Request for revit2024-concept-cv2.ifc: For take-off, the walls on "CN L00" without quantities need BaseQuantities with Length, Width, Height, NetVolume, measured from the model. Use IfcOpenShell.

First a look at what the model holds.

```python
import ifcopenshell
import ifcopenshell.util.element
import ifcopenshell.util.unit

model = ifcopenshell.open("revit2024-concept-cv2.ifc")
print(model.schema)
for unit_type in ("LENGTHUNIT", "AREAUNIT", "VOLUMEUNIT"):
    print(unit_type, ifcopenshell.util.unit.calculate_unit_scale(model, unit_type))
storey = next(s for s in model.by_type("IfcBuildingStorey") if s.Name == "CN L00")
walls = [e for e in ifcopenshell.util.element.get_decomposition(storey) if e.is_a("IfcWall")]
for e in sorted(walls, key=lambda e: e.id()):
    print(e.id(), e.is_a(), e.Name, list(ifcopenshell.util.element.get_psets(e, qtos_only=True)), sep=" | ")
```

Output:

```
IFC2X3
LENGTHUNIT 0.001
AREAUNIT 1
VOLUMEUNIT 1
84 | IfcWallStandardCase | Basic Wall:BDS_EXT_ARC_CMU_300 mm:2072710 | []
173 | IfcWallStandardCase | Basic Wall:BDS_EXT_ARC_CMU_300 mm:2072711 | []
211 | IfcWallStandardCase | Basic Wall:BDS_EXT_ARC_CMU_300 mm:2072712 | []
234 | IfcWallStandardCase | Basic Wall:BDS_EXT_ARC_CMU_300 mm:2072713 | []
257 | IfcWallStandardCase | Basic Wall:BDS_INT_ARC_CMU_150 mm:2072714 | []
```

```python
import ifcopenshell
import ifcopenshell.api.pset
import ifcopenshell.geom
import ifcopenshell.util.element
import ifcopenshell.util.shape
import ifcopenshell.util.unit

model = ifcopenshell.open("revit2024-concept-cv2.ifc")
unit_scale = ifcopenshell.util.unit.calculate_unit_scale(model)
volume_scale = ifcopenshell.util.unit.calculate_unit_scale(model, "VOLUMEUNIT")
settings = ifcopenshell.geom.settings()

storey = next(s for s in model.by_type("IfcBuildingStorey") if s.Name == "CN L00")
walls = [e for e in ifcopenshell.util.element.get_decomposition(storey) if e.is_a("IfcWall")]

for e in sorted(walls, key=lambda e: e.id()):
    if ifcopenshell.util.element.get_psets(e, qtos_only=True, should_inherit=False):
        continue
    # Geometry comes back in metres, in the element's own axes.
    shape = ifcopenshell.geom.create_shape(settings, e)
    values = {
        "Length": ifcopenshell.util.shape.get_x(shape.geometry) / unit_scale,
        "Width": ifcopenshell.util.shape.get_y(shape.geometry) / unit_scale,
        "Height": ifcopenshell.util.shape.get_z(shape.geometry) / unit_scale,
        "NetVolume": ifcopenshell.util.shape.get_volume(shape.geometry) / volume_scale,
    }
    qto = ifcopenshell.api.pset.add_qto(model, product=e, name="BaseQuantities")
    ifcopenshell.api.pset.edit_qto(model, qto=qto, properties=values)
    print(e.id(), {k: round(v, 3) for k, v in values.items()})

model.write("revit2024-concept-cv2-out.ifc")
```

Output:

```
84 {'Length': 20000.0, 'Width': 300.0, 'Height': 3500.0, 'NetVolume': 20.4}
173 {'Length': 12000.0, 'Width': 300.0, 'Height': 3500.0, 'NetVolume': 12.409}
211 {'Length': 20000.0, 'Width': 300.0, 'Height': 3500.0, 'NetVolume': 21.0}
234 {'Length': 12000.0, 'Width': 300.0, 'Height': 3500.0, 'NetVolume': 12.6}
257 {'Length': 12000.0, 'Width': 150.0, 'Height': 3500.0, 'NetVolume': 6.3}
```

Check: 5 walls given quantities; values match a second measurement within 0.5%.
